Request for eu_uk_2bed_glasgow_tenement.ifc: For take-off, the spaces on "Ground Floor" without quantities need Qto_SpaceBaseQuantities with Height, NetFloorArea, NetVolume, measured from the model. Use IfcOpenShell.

First a look at what the model holds.

```python
import ifcopenshell
import ifcopenshell.util.element
import ifcopenshell.util.unit

model = ifcopenshell.open("eu_uk_2bed_glasgow_tenement.ifc")
print(model.schema)
for unit_type in ("LENGTHUNIT", "AREAUNIT", "VOLUMEUNIT"):
    print(unit_type, ifcopenshell.util.unit.calculate_unit_scale(model, unit_type))
storey = next(s for s in model.by_type("IfcBuildingStorey") if s.Name == "Ground Floor")
spaces = [e for e in ifcopenshell.util.element.get_decomposition(storey) if e.is_a("IfcSpace")]
for e in sorted(spaces, key=lambda e: e.id()):
    print(e.id(), e.is_a(), e.Name, list(ifcopenshell.util.element.get_psets(e, qtos_only=True)), sep=" | ")
```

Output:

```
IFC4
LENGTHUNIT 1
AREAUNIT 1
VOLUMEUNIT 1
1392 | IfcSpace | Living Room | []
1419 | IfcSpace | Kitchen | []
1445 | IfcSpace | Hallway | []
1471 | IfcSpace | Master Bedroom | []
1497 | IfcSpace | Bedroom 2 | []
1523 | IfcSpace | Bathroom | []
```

```python
import ifcopenshell
import ifcopenshell.api.pset
import ifcopenshell.geom
import ifcopenshell.util.element
import ifcopenshell.util.shape
import ifcopenshell.util.unit

model = ifcopenshell.open("eu_uk_2bed_glasgow_tenement.ifc")
unit_scale = ifcopenshell.util.unit.calculate_unit_scale(model)
area_scale = ifcopenshell.util.unit.calculate_unit_scale(model, "AREAUNIT")
volume_scale = ifcopenshell.util.unit.calculate_unit_scale(model, "VOLUMEUNIT")
settings = ifcopenshell.geom.settings()

storey = next(s for s in model.by_type("IfcBuildingStorey") if s.Name == "Ground Floor")
spaces = [e for e in ifcopenshell.util.element.get_decomposition(storey) if e.is_a("IfcSpace")]

for e in sorted(spaces, key=lambda e: e.id()):
    if ifcopenshell.util.element.get_psets(e, qtos_only=True, should_inherit=False):
        continue
    # Geometry comes back in metres, in the element's own axes.
    shape = ifcopenshell.geom.create_shape(settings, e)
    values = {
        "Height": ifcopenshell.util.shape.get_z(shape.geometry) / unit_scale,
        "NetFloorArea": ifcopenshell.util.shape.get_footprint_area(shape.geometry) / area_scale,
        "NetVolume": ifcopenshell.util.shape.get_volume(shape.geometry) / volume_scale,
    }
    qto = ifcopenshell.api.pset.add_qto(model, product=e, name="Qto_SpaceBaseQuantities")
    ifcopenshell.api.pset.edit_qto(model, qto=qto, properties=values)
    print(e.id(), {k: round(v, 3) for k, v in values.items()})

model.write("eu_uk_2bed_glasgow_tenement-out.ifc")
```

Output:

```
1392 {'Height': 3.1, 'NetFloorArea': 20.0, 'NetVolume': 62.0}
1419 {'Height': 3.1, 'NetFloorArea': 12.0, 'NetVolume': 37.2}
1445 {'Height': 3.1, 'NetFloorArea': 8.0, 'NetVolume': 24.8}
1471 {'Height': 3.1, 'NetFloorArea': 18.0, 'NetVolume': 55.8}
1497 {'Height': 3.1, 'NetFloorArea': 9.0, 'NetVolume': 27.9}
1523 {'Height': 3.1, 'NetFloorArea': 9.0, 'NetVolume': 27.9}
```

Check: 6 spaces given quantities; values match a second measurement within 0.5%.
